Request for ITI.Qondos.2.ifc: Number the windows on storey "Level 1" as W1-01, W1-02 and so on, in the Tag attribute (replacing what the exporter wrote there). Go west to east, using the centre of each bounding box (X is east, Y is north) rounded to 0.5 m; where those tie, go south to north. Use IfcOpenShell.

First a look at what the model holds.

```python
import ifcopenshell
import ifcopenshell.util.element
import ifcopenshell.util.placement

model = ifcopenshell.open("ITI.Qondos.2.ifc")
print(model.schema)
storey = next(s for s in model.by_type("IfcBuildingStorey") if s.Name == "Level 1")
windows = [e for e in ifcopenshell.util.element.get_decomposition(storey) if e.is_a("IfcWindow")]
for e in sorted(windows, key=lambda e: e.id()):
    origin = ifcopenshell.util.placement.get_local_placement(e.ObjectPlacement)[:3, 3]
    print(e.id(), e.Tag, e.Name, origin.round(2) + 0.0, sep=" | ")
```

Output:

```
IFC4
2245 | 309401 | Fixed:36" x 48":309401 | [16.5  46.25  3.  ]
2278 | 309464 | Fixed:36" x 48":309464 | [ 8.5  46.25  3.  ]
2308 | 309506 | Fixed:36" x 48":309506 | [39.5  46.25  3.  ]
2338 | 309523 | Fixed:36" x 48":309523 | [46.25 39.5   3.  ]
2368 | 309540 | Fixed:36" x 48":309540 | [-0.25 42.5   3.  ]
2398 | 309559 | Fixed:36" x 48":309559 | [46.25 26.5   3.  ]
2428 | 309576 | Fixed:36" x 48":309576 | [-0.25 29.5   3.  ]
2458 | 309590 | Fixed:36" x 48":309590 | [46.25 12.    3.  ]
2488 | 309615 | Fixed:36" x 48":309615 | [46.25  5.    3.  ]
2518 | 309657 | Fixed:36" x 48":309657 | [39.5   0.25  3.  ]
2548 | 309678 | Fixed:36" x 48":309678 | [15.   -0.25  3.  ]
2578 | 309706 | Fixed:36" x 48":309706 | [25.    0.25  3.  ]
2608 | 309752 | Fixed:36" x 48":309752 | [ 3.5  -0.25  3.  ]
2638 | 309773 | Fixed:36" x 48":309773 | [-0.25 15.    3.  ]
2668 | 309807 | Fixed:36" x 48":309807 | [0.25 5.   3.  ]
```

```python
import ifcopenshell
import ifcopenshell.geom
import ifcopenshell.util.element
import ifcopenshell.util.shape

model = ifcopenshell.open("ITI.Qondos.2.ifc")
settings = ifcopenshell.geom.settings()
settings.set("use-world-coords", True)


def centre(element):
    shape = ifcopenshell.geom.create_shape(settings, element)
    return ifcopenshell.util.shape.get_bbox_centroid(shape.geometry)


storey = next(s for s in model.by_type("IfcBuildingStorey") if s.Name == "Level 1")
windows = [e for e in ifcopenshell.util.element.get_decomposition(storey) if e.is_a("IfcWindow")]

# Insertion points can sit at a corner or the storey origin, so sort by the geometry (in metres).
centres = {e: centre(e) for e in windows}
windows.sort(key=lambda e: (round(centres[e][0] / 0.5), centres[e][1]))

for i, e in enumerate(windows, start=1):
    number = f"W1-{i:02d}"
    e.Tag = number
    print(e.id(), number)

model.write("ITI.Qondos.2_edited.ifc")
```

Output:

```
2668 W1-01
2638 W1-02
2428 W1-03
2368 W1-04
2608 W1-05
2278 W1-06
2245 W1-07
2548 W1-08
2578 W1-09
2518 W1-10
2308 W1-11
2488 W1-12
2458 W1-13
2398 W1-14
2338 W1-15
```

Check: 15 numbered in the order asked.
